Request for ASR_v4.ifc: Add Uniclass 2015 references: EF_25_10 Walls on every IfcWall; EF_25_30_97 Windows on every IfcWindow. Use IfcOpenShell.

First a look at what the model holds.

```python
import ifcopenshell

model = ifcopenshell.open("ASR_v4.ifc")
print(model.schema)
print("classifications:", [c.Name for c in model.by_type("IfcClassification")])
for ifc_class in ("IfcDoor", "IfcRoof", "IfcStair", "IfcWall", "IfcWindow"):
    print(ifc_class, len(model.by_type(ifc_class)))
```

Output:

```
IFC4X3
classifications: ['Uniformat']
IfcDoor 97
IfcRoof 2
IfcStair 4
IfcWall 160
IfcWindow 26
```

```python
import ifcopenshell
import ifcopenshell.api.classification

model = ifcopenshell.open("ASR_v4.ifc")

system = ifcopenshell.api.classification.add_classification(model, classification="Uniclass 2015")

codes = {
    "IfcWall": ("EF_25_10", "Walls"),
    "IfcWindow": ("EF_25_30_97", "Windows"),
}
for ifc_class, (code, name) in codes.items():
    products = model.by_type(ifc_class)
    ifcopenshell.api.classification.add_reference(
        model, products=products, classification=system, identification=code, name=name
    )
    print(code, len(products))

model.write("ASR_v4_v2.ifc")
```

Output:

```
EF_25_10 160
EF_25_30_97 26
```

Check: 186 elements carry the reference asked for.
